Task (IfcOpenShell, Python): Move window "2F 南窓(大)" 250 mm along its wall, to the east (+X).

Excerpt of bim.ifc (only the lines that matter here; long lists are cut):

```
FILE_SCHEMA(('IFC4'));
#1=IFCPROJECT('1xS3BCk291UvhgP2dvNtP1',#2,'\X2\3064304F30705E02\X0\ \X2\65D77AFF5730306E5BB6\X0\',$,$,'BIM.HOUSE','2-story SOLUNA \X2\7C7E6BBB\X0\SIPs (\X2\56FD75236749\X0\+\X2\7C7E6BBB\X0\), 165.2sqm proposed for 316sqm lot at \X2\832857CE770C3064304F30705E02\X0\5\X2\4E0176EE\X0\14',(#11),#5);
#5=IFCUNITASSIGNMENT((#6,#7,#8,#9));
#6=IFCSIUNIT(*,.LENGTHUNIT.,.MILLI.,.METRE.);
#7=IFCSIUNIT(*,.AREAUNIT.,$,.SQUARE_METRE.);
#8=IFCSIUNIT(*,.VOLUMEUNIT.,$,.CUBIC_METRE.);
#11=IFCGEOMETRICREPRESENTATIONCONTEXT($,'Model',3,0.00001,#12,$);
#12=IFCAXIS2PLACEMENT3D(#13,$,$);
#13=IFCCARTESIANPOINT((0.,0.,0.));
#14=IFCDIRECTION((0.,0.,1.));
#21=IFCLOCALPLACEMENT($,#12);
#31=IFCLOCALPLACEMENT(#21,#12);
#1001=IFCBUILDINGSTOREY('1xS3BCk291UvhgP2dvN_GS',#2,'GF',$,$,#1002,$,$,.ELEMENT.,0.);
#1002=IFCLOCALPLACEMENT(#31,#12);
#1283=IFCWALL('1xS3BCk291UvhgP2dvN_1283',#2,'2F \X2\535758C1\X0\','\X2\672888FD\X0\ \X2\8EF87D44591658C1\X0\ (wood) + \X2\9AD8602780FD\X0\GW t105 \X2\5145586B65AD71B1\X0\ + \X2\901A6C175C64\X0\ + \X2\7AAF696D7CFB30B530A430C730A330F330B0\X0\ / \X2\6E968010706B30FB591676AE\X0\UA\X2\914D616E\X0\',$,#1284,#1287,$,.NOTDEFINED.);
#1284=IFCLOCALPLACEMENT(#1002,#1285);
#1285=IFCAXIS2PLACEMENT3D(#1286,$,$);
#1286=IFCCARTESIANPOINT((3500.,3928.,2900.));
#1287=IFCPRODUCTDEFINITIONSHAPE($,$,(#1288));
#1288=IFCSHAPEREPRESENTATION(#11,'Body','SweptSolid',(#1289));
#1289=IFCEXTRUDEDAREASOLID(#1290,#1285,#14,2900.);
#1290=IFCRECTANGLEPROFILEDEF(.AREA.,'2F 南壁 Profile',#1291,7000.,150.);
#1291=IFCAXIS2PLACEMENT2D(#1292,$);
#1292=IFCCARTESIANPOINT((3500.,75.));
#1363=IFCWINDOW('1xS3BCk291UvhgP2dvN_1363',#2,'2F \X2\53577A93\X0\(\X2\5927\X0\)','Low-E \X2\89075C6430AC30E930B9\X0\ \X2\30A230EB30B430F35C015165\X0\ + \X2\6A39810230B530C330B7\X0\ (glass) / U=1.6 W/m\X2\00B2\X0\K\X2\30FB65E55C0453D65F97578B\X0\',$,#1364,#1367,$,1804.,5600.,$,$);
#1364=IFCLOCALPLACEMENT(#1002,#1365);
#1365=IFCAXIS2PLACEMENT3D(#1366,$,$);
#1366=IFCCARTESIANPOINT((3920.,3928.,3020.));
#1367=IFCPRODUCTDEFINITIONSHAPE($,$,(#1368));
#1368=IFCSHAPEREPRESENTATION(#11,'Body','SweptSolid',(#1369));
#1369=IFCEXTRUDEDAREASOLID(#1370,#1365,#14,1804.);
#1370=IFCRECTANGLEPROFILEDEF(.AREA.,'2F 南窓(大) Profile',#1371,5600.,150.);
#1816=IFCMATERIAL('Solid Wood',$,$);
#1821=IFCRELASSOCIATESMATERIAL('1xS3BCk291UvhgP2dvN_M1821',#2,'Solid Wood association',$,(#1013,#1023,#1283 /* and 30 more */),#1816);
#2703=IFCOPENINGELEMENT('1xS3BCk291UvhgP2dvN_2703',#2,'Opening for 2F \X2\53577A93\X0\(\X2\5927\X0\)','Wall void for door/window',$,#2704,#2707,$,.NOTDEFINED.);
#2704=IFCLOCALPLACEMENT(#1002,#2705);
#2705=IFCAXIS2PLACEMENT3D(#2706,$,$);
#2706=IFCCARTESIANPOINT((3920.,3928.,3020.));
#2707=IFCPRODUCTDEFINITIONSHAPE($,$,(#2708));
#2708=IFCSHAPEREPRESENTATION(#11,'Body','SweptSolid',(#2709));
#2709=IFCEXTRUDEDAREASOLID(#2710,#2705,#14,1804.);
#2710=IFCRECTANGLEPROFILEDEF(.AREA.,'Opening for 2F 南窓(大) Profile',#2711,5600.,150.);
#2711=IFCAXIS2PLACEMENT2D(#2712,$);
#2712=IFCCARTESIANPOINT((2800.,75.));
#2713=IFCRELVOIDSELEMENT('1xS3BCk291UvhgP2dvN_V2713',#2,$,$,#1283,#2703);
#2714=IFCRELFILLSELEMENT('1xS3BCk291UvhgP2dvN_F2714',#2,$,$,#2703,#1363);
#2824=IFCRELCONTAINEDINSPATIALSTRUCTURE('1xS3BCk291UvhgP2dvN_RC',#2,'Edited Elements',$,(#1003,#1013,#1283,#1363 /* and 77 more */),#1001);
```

```python
import ifcopenshell
import ifcopenshell.api.geometry
import ifcopenshell.util.placement

model = ifcopenshell.open("bim.ifc")

window = model.by_id(1363)
opening = window.FillsVoids[0].RelatingOpeningElement
wall = opening.VoidsElements[0].RelatingBuildingElement

wall_matrix = ifcopenshell.util.placement.get_local_placement(wall.ObjectPlacement)
shift = wall_matrix[:3, 0] * 250.0
before = ifcopenshell.util.placement.get_local_placement(window.ObjectPlacement)[:3, 3].copy()

# The window is not placed relative to its opening, so move both.
for product in (opening, window):
    matrix = ifcopenshell.util.placement.get_local_placement(product.ObjectPlacement)
    matrix[:3, 3] += shift
    ifcopenshell.api.geometry.edit_object_placement(model, product=product, matrix=matrix, is_si=False)

after = ifcopenshell.util.placement.get_local_placement(window.ObjectPlacement)[:3, 3]
print("window moved by", (after - before).round(3) + 0.0)

model.write("bim_edited.ifc")
```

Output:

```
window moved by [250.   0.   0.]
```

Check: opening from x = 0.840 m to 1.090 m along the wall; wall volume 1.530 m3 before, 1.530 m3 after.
